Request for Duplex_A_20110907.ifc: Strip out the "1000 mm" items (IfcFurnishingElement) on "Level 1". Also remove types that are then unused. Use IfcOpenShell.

First a look at what the model holds.

```python
import ifcopenshell
import ifcopenshell.util.element

model = ifcopenshell.open("Duplex_A_20110907.ifc")
print(model.schema)
storey = next(s for s in model.by_type("IfcBuildingStorey") if s.Name == "Level 1")
furniture = [e for e in ifcopenshell.util.element.get_decomposition(storey) if e.is_a("IfcFurnishingElement")]
seen = {}
for e in furniture:
    element_type = ifcopenshell.util.element.get_type(e)
    name = element_type.Name if element_type not in (None, e) else None
    seen[name] = seen.get(name, 0) + 1
for name, count in sorted(seen.items(), key=str):
    print(count, "x", name)
```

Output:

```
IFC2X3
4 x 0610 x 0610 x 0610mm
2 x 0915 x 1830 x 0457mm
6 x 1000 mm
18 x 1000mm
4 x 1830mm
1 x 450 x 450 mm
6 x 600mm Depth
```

```python
import ifcopenshell
import ifcopenshell.api.root
import ifcopenshell.util.element

model = ifcopenshell.open("Duplex_A_20110907.ifc")

storey = next(s for s in model.by_type("IfcBuildingStorey") if s.Name == "Level 1")
furniture = [e for e in ifcopenshell.util.element.get_decomposition(storey) if e.is_a("IfcFurnishingElement")]
targets = [e for e in furniture if (t := ifcopenshell.util.element.get_type(e)) not in (None, e) and t.Name == "1000 mm"]
types = {ifcopenshell.util.element.get_type(e) for e in targets} - {None, *targets}

for e in targets:
    ifcopenshell.api.root.remove_product(model, product=e)
print(len(targets), "removed")

unused = [t for t in types if not ifcopenshell.util.element.get_types(t)]
for t in unused:
    ifcopenshell.api.root.remove_product(model, product=t)
print(len(unused), "unused types removed")

model.write("Duplex_A_20110907_updated.ifc")
```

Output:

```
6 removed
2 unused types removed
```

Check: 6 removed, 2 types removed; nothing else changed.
